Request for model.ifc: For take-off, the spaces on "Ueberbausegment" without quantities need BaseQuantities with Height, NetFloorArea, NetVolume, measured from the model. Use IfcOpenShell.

First a look at what the model holds.

```python
import ifcopenshell
import ifcopenshell.util.element
import ifcopenshell.util.unit

model = ifcopenshell.open("model.ifc")
print(model.schema)
for unit_type in ("LENGTHUNIT", "AREAUNIT", "VOLUMEUNIT"):
    print(unit_type, ifcopenshell.util.unit.calculate_unit_scale(model, unit_type))
storey = next(s for s in model.by_type("IfcBuildingStorey") if s.Name == "Ueberbausegment")
spaces = [e for e in ifcopenshell.util.element.get_decomposition(storey) if e.is_a("IfcSpace")]
for e in sorted(spaces, key=lambda e: e.id()):
    print(e.id(), e.is_a(), e.Name, list(ifcopenshell.util.element.get_psets(e, qtos_only=True)), sep=" | ")
```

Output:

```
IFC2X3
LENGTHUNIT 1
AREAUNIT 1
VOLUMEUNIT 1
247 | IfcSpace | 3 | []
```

```python
import ifcopenshell
import ifcopenshell.api.pset
import ifcopenshell.geom
import ifcopenshell.util.element
import ifcopenshell.util.shape
import ifcopenshell.util.unit

model = ifcopenshell.open("model.ifc")
unit_scale = ifcopenshell.util.unit.calculate_unit_scale(model)
area_scale = ifcopenshell.util.unit.calculate_unit_scale(model, "AREAUNIT")
volume_scale = ifcopenshell.util.unit.calculate_unit_scale(model, "VOLUMEUNIT")
settings = ifcopenshell.geom.settings()

storey = next(s for s in model.by_type("IfcBuildingStorey") if s.Name == "Ueberbausegment")
spaces = [e for e in ifcopenshell.util.element.get_decomposition(storey) if e.is_a("IfcSpace")]

for e in sorted(spaces, key=lambda e: e.id()):
    if ifcopenshell.util.element.get_psets(e, qtos_only=True, should_inherit=False):
        continue
    # Geometry comes back in metres, in the element's own axes.
    shape = ifcopenshell.geom.create_shape(settings, e)
    values = {
        "Height": ifcopenshell.util.shape.get_z(shape.geometry) / unit_scale,
        "NetFloorArea": ifcopenshell.util.shape.get_footprint_area(shape.geometry) / area_scale,
        "NetVolume": ifcopenshell.util.shape.get_volume(shape.geometry) / volume_scale,
    }
    qto = ifcopenshell.api.pset.add_qto(model, product=e, name="BaseQuantities")
    ifcopenshell.api.pset.edit_qto(model, qto=qto, properties=values)
    print(e.id(), {k: round(v, 3) for k, v in values.items()})

model.write("model_v2.ifc")
```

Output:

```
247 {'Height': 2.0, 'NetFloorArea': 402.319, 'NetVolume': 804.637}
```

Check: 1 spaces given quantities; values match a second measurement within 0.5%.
